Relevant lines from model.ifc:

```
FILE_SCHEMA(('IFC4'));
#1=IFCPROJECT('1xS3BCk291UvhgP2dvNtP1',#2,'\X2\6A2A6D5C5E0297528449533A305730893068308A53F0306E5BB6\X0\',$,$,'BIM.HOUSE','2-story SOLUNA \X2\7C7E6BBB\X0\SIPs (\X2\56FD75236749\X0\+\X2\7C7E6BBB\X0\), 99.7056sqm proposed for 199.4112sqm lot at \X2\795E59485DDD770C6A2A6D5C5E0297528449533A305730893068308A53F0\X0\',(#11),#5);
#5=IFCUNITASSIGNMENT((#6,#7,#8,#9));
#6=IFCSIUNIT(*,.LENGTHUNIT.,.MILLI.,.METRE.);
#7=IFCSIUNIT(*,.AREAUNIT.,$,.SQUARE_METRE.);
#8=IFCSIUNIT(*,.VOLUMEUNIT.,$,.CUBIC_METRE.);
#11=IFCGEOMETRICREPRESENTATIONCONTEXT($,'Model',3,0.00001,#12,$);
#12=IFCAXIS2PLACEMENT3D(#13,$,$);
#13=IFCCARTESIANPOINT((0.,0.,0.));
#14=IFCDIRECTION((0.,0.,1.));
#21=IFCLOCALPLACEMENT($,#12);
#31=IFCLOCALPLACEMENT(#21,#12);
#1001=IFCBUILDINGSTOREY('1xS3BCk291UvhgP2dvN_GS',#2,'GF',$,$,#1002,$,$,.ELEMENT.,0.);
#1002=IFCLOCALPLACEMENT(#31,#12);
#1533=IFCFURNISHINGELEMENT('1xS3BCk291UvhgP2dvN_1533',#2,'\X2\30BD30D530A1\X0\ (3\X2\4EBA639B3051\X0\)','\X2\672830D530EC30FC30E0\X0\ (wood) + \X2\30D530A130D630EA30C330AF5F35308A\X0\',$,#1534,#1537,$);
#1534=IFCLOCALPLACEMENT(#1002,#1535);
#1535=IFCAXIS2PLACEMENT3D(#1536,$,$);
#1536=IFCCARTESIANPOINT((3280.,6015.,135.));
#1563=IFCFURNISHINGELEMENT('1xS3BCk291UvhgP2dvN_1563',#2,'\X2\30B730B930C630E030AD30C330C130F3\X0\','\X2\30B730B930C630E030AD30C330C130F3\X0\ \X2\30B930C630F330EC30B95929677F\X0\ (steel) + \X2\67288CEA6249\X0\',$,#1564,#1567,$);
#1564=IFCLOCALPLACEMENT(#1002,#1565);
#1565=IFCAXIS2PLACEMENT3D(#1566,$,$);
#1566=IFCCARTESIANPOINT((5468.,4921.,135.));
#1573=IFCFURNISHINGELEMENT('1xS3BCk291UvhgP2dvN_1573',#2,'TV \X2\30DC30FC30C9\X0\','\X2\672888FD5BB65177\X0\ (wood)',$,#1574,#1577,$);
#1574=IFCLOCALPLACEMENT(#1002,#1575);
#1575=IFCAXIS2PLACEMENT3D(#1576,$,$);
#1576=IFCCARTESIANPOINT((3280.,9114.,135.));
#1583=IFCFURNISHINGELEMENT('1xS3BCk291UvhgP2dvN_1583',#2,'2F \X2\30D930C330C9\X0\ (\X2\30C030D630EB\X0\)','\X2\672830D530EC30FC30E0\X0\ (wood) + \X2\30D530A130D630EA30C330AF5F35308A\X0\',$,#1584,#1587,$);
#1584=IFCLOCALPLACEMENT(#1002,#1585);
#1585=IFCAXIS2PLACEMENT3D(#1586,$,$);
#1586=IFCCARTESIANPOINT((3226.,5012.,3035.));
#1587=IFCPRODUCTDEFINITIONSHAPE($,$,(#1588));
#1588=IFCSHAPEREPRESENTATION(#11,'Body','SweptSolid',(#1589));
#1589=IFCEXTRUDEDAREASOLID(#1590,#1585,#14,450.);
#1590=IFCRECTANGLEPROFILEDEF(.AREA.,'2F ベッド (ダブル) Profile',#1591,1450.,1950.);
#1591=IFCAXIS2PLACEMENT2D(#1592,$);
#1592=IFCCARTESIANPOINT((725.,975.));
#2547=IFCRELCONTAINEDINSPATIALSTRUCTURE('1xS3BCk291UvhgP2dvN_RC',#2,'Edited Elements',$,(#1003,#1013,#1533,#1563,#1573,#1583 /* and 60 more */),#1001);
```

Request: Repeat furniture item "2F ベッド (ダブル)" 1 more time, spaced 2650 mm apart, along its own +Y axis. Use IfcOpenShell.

```python
import ifcopenshell
import ifcopenshell.api.geometry
import ifcopenshell.api.root
import ifcopenshell.util.element
import ifcopenshell.util.placement

model = ifcopenshell.open("model.ifc")


def reuse_history(source, copy):
    """copy_class also copies each property set's owner history, people and application; keep the originals."""
    for rel in copy.IsDefinedBy:
        if rel.is_a("IfcRelDefinesByProperties") and (history := rel.RelatingPropertyDefinition.OwnerHistory):
            rel.RelatingPropertyDefinition.OwnerHistory = source.OwnerHistory
            ifcopenshell.util.element.remove_deep2(model, history)


source = model.by_guid("1xS3BCk291UvhgP2dvN_1583")
base = ifcopenshell.util.placement.get_local_placement(source.ObjectPlacement)
step = base[:3, 1] * 2650.0

for i in range(1, 2):
    copy = ifcopenshell.api.root.copy_class(model, product=source)
    copy.Representation = ifcopenshell.util.element.copy_deep(
        model, source.Representation, exclude=["IfcGeometricRepresentationContext", "IfcRepresentationMap"]
    )
    reuse_history(source, copy)
    matrix = base.copy()
    matrix[:3, 3] += i * step
    print("added at", matrix[:3, 3].round(3) + 0.0)
    ifcopenshell.api.geometry.edit_object_placement(model, product=copy, matrix=matrix, is_si=False)

model.write("model-out.ifc")
```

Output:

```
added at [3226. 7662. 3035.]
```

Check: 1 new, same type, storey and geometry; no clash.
